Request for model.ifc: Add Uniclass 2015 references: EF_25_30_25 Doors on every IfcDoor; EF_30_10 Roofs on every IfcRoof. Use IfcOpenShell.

First a look at what the model holds.

```python
import ifcopenshell

model = ifcopenshell.open("model.ifc")
print(model.schema)
print("classifications:", [c.Name for c in model.by_type("IfcClassification")])
for ifc_class in ("IfcDoor", "IfcRoof", "IfcStair", "IfcWall", "IfcWindow"):
    print(ifc_class, len(model.by_type(ifc_class)))
```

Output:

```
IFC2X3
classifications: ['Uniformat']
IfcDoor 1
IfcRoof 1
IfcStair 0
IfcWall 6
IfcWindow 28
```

```python
import ifcopenshell
import ifcopenshell.api.classification

model = ifcopenshell.open("model.ifc")

# IFC2X3 requires Source and Edition and has no link from the project to the system.
system = model.create_entity("IfcClassification", Source="NBS", Edition="2015", Name="Uniclass 2015")

codes = {
    "IfcDoor": ("EF_25_30_25", "Doors"),
    "IfcRoof": ("EF_30_10", "Roofs"),
}
for ifc_class, (code, name) in codes.items():
    products = model.by_type(ifc_class)
    ifcopenshell.api.classification.add_reference(
        model, products=products, classification=system, identification=code, name=name
    )
    print(code, len(products))

model.write("model_rev.ifc")
```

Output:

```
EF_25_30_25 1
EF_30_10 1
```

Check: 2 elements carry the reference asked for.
